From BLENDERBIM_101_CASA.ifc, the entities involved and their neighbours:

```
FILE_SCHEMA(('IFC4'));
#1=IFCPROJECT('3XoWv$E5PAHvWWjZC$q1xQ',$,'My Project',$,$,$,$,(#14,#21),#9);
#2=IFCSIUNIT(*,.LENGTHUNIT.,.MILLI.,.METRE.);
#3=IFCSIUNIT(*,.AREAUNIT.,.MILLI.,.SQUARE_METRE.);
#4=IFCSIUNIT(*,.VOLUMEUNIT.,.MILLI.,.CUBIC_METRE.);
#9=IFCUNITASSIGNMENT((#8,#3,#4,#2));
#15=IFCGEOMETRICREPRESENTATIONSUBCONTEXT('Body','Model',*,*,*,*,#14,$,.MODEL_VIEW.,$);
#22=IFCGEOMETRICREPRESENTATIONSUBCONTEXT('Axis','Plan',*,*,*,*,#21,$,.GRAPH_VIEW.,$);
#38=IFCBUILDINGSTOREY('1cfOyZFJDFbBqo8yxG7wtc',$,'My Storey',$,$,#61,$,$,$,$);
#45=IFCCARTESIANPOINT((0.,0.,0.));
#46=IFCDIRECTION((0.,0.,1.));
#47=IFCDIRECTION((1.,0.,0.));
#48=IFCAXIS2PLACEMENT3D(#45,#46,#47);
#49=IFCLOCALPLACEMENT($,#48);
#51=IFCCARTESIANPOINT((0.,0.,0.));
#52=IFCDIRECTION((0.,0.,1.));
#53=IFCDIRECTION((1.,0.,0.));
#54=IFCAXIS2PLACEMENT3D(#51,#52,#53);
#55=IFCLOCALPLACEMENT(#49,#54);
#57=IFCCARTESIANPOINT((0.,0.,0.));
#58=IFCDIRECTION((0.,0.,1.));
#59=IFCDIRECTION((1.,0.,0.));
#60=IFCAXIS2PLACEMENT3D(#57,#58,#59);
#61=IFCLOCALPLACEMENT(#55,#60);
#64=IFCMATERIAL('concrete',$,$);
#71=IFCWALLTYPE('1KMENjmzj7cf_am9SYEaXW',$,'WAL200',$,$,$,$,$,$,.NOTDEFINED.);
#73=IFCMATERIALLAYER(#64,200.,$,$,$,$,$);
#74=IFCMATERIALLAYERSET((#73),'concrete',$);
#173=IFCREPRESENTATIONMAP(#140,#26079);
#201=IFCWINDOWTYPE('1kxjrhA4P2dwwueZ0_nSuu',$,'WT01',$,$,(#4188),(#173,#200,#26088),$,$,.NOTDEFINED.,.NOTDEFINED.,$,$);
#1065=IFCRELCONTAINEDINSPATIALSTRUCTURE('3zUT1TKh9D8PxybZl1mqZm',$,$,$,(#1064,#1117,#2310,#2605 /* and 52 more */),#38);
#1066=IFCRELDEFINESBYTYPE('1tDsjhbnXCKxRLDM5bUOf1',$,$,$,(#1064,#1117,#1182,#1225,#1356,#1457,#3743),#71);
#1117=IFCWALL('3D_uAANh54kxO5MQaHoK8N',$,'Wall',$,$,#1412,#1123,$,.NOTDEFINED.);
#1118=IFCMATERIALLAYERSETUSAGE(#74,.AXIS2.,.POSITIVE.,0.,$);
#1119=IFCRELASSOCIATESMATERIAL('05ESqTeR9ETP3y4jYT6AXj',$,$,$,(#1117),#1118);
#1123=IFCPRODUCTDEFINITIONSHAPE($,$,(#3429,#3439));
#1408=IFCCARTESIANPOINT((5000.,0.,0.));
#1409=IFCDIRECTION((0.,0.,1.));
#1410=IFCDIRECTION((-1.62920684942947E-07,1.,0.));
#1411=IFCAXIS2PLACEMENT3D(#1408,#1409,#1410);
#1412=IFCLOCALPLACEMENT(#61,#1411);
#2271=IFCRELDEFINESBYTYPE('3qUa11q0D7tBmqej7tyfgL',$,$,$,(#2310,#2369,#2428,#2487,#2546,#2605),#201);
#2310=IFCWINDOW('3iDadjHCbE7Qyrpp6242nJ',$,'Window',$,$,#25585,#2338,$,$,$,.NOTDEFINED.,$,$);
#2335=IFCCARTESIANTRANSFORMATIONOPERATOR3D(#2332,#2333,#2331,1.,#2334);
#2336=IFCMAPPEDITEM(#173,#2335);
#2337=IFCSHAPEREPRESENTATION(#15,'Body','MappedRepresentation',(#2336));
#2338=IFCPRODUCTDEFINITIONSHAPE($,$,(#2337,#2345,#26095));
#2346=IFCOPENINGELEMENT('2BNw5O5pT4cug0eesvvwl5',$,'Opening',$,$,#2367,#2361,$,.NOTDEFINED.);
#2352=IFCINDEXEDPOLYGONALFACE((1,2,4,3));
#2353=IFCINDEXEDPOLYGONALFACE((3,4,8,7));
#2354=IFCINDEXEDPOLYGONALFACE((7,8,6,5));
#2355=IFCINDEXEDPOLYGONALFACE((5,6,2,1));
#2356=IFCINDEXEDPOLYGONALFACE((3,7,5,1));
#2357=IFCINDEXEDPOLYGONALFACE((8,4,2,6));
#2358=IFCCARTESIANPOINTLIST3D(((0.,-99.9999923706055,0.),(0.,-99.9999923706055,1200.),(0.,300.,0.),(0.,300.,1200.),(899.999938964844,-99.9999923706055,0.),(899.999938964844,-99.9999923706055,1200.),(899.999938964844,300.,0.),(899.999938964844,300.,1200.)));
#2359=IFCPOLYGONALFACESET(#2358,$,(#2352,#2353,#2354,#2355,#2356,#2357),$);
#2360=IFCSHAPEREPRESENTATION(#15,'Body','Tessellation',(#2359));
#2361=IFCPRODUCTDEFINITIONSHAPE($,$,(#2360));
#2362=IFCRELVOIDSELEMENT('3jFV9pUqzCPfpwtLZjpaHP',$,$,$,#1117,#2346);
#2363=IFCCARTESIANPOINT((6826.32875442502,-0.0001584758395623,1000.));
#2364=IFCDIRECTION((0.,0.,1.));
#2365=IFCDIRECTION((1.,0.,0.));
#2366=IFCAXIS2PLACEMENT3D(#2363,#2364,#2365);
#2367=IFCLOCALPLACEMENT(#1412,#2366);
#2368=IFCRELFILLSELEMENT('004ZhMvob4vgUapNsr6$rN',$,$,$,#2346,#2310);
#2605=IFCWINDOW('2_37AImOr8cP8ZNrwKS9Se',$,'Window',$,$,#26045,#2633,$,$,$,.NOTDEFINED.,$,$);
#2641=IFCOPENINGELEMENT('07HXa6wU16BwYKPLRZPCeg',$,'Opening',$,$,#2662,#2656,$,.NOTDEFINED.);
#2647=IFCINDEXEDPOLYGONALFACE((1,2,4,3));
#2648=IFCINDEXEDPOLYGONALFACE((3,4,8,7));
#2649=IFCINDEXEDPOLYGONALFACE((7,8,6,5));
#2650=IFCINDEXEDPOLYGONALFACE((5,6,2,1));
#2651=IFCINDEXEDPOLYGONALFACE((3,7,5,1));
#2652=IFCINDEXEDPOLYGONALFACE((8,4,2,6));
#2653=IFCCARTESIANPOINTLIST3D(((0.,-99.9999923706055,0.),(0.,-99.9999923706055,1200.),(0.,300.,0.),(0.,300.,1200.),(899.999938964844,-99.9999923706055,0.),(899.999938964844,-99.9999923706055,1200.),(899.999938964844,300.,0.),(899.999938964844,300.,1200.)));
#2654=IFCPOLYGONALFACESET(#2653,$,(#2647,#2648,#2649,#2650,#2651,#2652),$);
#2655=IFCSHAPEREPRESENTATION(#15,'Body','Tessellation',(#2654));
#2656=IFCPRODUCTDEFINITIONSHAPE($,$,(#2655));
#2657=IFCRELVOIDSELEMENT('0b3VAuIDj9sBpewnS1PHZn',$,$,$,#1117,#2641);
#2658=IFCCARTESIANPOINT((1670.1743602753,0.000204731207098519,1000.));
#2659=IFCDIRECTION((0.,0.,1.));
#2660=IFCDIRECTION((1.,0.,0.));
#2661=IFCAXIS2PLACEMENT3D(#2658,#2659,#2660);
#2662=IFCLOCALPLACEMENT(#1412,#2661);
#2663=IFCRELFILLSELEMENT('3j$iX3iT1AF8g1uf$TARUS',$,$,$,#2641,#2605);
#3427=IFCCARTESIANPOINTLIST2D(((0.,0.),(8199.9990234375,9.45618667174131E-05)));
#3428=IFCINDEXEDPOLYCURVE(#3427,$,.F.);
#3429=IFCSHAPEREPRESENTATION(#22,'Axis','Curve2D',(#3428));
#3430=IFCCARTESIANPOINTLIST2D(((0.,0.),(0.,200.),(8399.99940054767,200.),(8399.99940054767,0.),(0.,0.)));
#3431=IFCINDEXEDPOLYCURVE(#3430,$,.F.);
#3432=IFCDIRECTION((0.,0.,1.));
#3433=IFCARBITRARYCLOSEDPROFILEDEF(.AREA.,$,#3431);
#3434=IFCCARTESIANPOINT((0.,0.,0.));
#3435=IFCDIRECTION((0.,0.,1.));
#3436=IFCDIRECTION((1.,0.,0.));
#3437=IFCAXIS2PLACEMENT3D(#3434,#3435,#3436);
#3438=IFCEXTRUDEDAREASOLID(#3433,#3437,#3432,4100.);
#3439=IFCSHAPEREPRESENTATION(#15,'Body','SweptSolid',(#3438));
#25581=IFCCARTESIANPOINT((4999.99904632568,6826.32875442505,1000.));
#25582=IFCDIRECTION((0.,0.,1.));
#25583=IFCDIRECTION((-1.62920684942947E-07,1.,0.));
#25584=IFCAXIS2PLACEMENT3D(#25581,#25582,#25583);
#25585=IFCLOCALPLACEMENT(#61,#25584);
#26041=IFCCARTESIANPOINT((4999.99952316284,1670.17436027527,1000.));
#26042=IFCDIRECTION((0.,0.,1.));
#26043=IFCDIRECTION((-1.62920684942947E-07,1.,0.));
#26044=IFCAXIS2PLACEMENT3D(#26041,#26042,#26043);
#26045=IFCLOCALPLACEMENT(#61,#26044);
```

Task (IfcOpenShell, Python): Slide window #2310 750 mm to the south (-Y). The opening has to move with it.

```python
import ifcopenshell
import ifcopenshell.api.geometry
import ifcopenshell.util.placement
import ifcopenshell.util.unit

model = ifcopenshell.open("BLENDERBIM_101_CASA.ifc")
unit_scale = ifcopenshell.util.unit.calculate_unit_scale(model)

window = model.by_guid("3iDadjHCbE7Qyrpp6242nJ")
opening = window.FillsVoids[0].RelatingOpeningElement
wall = opening.VoidsElements[0].RelatingBuildingElement

wall_matrix = ifcopenshell.util.placement.get_local_placement(wall.ObjectPlacement)
shift = wall_matrix[:3, 0] * -0.75 / unit_scale
before = ifcopenshell.util.placement.get_local_placement(window.ObjectPlacement)[:3, 3].copy()

# The window is not placed relative to its opening, so move both.
for product in (opening, window):
    matrix = ifcopenshell.util.placement.get_local_placement(product.ObjectPlacement)
    matrix[:3, 3] += shift
    ifcopenshell.api.geometry.edit_object_placement(model, product=product, matrix=matrix, is_si=False)

after = ifcopenshell.util.placement.get_local_placement(window.ObjectPlacement)[:3, 3]
print("window moved by", (after - before).round(3) + 0.0)

model.write("BLENDERBIM_101_CASA_rev.ifc")
```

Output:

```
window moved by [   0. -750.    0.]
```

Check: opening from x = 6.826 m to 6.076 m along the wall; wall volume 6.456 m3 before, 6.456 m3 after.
